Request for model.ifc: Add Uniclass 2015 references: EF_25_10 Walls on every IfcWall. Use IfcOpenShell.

First a look at what the model holds.

```python
import ifcopenshell

model = ifcopenshell.open("model.ifc")
print(model.schema)
print("classifications:", [c.Name for c in model.by_type("IfcClassification")])
for ifc_class in ("IfcDoor", "IfcRoof", "IfcStair", "IfcWall", "IfcWindow"):
    print(ifc_class, len(model.by_type(ifc_class)))
```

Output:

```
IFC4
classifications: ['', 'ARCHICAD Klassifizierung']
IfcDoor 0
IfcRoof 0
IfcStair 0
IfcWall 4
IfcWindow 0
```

```python
import ifcopenshell
import ifcopenshell.api.classification

model = ifcopenshell.open("model.ifc")

system = ifcopenshell.api.classification.add_classification(model, classification="Uniclass 2015")

codes = {
    "IfcWall": ("EF_25_10", "Walls"),
}
for ifc_class, (code, name) in codes.items():
    products = model.by_type(ifc_class)
    ifcopenshell.api.classification.add_reference(
        model, products=products, classification=system, identification=code, name=name
    )
    print(code, len(products))

model.write("model_rev.ifc")
```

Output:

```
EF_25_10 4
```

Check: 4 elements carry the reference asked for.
